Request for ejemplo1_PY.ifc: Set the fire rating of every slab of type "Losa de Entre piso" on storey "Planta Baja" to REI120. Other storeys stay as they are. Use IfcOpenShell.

First a look at what the model holds.

```python
import ifcopenshell
import ifcopenshell.util.element

model = ifcopenshell.open("ejemplo1_PY.ifc")
print(model.schema)
storey = next(s for s in model.by_type("IfcBuildingStorey") if s.Name == "Planta Baja")
slabs = [e for e in ifcopenshell.util.element.get_decomposition(storey) if e.is_a("IfcSlab")]
seen = {}
for e in slabs:
    element_type = ifcopenshell.util.element.get_type(e)
    key = (element_type.Name if element_type != e and element_type else None, ifcopenshell.util.element.get_pset(e, "Pset_SlabCommon", "FireRating"))
    seen[key] = seen.get(key, 0) + 1
for (name, value), count in sorted(seen.items(), key=str):
    print(count, "x", name, "|", value)
```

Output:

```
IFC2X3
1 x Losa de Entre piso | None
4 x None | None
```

```python
import ifcopenshell
import ifcopenshell.api.pset
import ifcopenshell.util.element

model = ifcopenshell.open("ejemplo1_PY.ifc")

storey = next(s for s in model.by_type("IfcBuildingStorey") if s.Name == "Planta Baja")
slabs = [e for e in ifcopenshell.util.element.get_decomposition(storey) if e.is_a("IfcSlab")]

count = 0
for e in slabs:
    element_type = ifcopenshell.util.element.get_type(e)
    if element_type in (None, e) or element_type.Name != "Losa de Entre piso":
        continue
    # add_pset returns the element's existing set when there is one.
    pset = ifcopenshell.api.pset.add_pset(model, product=e, name="Pset_SlabCommon")
    ifcopenshell.api.pset.edit_pset(model, pset=pset, properties={"FireRating": "REI120"})
    count += 1

print(count, "slabs updated")

model.write("ejemplo1_PY_updated.ifc")
```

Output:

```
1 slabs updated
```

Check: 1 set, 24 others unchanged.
